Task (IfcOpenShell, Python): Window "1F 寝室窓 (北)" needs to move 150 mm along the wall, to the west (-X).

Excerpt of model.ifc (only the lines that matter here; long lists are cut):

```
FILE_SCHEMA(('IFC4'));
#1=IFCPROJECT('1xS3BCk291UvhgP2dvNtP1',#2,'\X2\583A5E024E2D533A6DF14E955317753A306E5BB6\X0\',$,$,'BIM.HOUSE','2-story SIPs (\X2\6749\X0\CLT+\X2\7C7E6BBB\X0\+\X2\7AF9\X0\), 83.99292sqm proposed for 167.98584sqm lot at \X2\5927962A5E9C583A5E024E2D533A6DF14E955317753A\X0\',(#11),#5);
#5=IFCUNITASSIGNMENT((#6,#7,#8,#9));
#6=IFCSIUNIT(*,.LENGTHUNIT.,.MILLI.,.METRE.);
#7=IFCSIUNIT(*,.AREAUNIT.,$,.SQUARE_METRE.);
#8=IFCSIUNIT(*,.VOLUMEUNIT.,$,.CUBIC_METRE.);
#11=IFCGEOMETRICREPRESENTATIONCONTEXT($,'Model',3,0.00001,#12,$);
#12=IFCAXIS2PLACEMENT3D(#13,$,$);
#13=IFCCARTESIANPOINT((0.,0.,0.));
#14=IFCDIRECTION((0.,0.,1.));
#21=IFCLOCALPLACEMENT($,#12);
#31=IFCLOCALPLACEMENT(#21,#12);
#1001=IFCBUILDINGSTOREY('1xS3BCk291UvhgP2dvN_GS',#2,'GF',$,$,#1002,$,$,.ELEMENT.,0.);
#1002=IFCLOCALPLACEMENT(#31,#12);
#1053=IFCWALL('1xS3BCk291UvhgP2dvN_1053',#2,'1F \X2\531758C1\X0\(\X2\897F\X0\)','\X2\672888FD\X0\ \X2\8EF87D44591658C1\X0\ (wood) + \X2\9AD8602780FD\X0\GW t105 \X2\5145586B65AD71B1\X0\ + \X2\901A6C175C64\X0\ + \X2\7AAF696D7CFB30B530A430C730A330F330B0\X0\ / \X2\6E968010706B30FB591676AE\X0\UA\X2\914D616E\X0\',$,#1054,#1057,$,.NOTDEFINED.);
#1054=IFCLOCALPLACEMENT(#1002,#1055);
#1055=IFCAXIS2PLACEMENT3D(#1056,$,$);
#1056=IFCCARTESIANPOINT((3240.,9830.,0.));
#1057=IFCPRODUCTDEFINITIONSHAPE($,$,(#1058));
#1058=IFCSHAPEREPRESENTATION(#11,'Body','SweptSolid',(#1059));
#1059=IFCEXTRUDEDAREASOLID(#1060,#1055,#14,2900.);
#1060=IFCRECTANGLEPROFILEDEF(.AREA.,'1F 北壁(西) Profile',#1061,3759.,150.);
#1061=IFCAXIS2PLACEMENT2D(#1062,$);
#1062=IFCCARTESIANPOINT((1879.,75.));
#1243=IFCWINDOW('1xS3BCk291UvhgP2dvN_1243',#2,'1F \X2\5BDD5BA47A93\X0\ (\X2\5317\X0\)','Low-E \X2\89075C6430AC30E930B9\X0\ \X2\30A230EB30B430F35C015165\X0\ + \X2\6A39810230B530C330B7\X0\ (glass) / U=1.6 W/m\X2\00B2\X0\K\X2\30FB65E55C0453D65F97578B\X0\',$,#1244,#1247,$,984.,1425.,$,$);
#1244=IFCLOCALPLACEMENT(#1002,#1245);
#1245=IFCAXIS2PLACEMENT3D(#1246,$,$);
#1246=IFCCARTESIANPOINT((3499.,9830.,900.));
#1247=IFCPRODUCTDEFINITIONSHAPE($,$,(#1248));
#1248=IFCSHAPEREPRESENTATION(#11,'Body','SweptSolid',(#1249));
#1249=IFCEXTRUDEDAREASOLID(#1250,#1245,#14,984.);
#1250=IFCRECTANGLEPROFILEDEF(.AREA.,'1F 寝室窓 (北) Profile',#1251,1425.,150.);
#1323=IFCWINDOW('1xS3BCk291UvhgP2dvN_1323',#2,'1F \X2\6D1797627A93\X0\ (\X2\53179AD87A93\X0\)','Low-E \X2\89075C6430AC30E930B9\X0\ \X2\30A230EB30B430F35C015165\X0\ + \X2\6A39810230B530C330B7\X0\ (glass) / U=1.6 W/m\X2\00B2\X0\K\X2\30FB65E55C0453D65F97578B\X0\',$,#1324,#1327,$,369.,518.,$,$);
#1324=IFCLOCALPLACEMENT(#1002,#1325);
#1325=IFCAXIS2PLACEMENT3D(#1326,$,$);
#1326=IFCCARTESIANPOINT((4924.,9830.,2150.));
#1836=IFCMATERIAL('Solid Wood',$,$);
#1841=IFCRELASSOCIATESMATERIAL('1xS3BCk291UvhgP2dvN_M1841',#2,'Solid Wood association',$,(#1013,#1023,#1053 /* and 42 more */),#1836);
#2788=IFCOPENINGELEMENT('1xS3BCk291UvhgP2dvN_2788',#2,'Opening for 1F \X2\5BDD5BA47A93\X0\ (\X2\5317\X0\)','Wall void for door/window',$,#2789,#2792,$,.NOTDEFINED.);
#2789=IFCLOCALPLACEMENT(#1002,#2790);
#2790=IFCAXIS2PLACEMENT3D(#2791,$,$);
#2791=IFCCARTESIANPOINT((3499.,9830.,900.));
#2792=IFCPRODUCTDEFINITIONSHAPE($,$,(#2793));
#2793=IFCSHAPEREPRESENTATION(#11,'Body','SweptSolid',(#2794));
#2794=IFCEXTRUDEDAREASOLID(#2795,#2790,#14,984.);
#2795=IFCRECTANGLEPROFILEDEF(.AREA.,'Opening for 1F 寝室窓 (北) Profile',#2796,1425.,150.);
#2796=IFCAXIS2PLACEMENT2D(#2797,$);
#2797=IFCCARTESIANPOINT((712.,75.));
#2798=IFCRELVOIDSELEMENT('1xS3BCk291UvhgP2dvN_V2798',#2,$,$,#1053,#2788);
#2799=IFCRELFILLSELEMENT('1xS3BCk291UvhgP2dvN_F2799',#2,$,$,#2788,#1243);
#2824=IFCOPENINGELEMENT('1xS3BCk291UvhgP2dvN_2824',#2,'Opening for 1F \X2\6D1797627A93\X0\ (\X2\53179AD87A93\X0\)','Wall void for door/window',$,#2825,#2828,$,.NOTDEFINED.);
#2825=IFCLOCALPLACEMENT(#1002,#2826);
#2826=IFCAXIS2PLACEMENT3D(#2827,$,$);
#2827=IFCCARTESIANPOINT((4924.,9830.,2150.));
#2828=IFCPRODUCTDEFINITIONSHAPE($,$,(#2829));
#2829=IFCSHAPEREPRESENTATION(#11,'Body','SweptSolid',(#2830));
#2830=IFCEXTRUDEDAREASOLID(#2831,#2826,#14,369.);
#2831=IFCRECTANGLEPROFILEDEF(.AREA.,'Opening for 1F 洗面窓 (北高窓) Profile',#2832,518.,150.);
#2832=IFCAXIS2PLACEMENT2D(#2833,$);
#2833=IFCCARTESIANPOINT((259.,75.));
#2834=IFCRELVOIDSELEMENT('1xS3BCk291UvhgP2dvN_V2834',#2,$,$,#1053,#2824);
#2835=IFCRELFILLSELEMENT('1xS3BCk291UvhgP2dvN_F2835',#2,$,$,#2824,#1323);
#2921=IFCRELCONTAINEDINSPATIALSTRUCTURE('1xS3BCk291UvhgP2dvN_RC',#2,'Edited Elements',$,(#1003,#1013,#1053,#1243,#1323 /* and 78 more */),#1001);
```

```python
import ifcopenshell
import ifcopenshell.api.geometry
import ifcopenshell.util.placement

model = ifcopenshell.open("model.ifc")

window = model.by_guid("1xS3BCk291UvhgP2dvN_1243")
opening = window.FillsVoids[0].RelatingOpeningElement
wall = opening.VoidsElements[0].RelatingBuildingElement

wall_matrix = ifcopenshell.util.placement.get_local_placement(wall.ObjectPlacement)
shift = wall_matrix[:3, 0] * -150.0
before = ifcopenshell.util.placement.get_local_placement(window.ObjectPlacement)[:3, 3].copy()

# The window is not placed relative to its opening, so move both.
for product in (opening, window):
    matrix = ifcopenshell.util.placement.get_local_placement(product.ObjectPlacement)
    matrix[:3, 3] += shift
    ifcopenshell.api.geometry.edit_object_placement(model, product=product, matrix=matrix, is_si=False)

after = ifcopenshell.util.placement.get_local_placement(window.ObjectPlacement)[:3, 3]
print("window moved by", (after - before).round(3) + 0.0)

model.write("model_updated.ifc")
```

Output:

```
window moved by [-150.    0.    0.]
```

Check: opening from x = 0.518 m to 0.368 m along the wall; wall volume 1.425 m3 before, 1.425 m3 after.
